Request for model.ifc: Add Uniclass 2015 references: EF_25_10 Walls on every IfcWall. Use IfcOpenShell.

First a look at what the model holds.

```python
import ifcopenshell

model = ifcopenshell.open("model.ifc")
print(model.schema)
print("classifications:", [c.Name for c in model.by_type("IfcClassification")])
for ifc_class in ("IfcDoor", "IfcRoof", "IfcStair", "IfcWall", "IfcWindow"):
    print(ifc_class, len(model.by_type(ifc_class)))
```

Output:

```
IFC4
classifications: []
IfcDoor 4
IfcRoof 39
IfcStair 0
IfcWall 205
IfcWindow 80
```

```python
import ifcopenshell
import ifcopenshell.api.classification

model = ifcopenshell.open("model.ifc")

system = ifcopenshell.api.classification.add_classification(model, classification="Uniclass 2015")

codes = {
    "IfcWall": ("EF_25_10", "Walls"),
}
for ifc_class, (code, name) in codes.items():
    products = model.by_type(ifc_class)
    ifcopenshell.api.classification.add_reference(
        model, products=products, classification=system, identification=code, name=name
    )
    print(code, len(products))

model.write("model-out.ifc")
```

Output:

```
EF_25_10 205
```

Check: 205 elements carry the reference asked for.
